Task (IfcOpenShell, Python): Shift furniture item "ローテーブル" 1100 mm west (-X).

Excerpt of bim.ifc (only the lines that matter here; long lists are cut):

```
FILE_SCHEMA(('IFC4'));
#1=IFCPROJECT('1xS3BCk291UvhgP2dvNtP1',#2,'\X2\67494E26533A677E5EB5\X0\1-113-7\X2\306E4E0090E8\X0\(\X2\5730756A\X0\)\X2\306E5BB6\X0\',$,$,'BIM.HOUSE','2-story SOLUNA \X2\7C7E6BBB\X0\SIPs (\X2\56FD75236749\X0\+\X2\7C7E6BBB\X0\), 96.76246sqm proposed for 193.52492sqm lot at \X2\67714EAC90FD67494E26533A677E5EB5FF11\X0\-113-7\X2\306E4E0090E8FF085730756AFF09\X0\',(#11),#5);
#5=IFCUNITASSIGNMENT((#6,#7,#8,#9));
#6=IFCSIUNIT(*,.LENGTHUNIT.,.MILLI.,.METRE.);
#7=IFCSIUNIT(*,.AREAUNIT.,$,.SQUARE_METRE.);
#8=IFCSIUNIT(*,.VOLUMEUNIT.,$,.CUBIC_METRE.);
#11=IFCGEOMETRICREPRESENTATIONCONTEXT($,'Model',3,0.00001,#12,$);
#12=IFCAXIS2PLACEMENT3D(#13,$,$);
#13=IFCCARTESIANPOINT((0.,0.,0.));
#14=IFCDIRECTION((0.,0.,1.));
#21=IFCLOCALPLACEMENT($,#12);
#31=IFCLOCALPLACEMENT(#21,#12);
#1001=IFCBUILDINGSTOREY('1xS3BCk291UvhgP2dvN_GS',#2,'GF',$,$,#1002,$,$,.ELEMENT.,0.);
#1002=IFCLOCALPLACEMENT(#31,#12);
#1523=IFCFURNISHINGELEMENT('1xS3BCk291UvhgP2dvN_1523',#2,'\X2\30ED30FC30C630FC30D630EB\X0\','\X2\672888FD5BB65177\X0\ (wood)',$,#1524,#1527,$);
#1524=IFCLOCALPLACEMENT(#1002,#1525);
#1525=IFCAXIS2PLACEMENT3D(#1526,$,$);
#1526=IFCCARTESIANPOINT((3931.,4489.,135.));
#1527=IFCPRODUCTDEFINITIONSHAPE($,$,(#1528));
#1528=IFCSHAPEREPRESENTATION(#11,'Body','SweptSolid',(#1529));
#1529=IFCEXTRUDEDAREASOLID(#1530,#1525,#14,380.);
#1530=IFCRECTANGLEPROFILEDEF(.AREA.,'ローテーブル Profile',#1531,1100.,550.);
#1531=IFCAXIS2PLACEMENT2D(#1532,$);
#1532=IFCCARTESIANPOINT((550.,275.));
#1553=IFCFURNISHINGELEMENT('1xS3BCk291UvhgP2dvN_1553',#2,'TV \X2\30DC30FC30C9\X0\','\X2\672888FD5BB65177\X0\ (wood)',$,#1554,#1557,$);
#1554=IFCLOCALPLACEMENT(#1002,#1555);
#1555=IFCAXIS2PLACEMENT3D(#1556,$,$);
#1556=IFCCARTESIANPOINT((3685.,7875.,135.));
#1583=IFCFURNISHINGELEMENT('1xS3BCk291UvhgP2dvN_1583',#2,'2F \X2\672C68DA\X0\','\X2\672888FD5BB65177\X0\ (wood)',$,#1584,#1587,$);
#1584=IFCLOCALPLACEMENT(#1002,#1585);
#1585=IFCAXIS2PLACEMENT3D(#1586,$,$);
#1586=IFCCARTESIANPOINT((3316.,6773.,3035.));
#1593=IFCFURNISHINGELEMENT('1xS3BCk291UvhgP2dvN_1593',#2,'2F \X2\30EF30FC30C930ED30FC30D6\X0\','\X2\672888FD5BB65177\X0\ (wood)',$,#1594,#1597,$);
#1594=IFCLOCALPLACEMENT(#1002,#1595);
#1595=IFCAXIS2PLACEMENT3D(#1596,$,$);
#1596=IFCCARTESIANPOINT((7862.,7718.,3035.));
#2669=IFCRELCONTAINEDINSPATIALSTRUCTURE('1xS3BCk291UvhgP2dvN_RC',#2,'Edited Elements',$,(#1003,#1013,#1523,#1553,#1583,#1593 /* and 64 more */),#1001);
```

```python
import ifcopenshell
import ifcopenshell.api.geometry
import ifcopenshell.util.placement
import ifcopenshell.util.unit

model = ifcopenshell.open("bim.ifc")
unit_scale = ifcopenshell.util.unit.calculate_unit_scale(model)

item = model.by_guid("1xS3BCk291UvhgP2dvN_1523")
matrix = ifcopenshell.util.placement.get_local_placement(item.ObjectPlacement)
matrix[0, 3] -= 1.1 / unit_scale
ifcopenshell.api.geometry.edit_object_placement(model, product=item, matrix=matrix, is_si=False)

print(ifcopenshell.util.placement.get_local_placement(item.ObjectPlacement).round(3) + 0.0)

model.write("bim_rev.ifc")
```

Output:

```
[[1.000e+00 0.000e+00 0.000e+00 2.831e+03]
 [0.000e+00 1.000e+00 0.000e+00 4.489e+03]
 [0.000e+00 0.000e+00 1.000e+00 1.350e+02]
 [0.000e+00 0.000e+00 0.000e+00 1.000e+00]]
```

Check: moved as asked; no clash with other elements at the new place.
